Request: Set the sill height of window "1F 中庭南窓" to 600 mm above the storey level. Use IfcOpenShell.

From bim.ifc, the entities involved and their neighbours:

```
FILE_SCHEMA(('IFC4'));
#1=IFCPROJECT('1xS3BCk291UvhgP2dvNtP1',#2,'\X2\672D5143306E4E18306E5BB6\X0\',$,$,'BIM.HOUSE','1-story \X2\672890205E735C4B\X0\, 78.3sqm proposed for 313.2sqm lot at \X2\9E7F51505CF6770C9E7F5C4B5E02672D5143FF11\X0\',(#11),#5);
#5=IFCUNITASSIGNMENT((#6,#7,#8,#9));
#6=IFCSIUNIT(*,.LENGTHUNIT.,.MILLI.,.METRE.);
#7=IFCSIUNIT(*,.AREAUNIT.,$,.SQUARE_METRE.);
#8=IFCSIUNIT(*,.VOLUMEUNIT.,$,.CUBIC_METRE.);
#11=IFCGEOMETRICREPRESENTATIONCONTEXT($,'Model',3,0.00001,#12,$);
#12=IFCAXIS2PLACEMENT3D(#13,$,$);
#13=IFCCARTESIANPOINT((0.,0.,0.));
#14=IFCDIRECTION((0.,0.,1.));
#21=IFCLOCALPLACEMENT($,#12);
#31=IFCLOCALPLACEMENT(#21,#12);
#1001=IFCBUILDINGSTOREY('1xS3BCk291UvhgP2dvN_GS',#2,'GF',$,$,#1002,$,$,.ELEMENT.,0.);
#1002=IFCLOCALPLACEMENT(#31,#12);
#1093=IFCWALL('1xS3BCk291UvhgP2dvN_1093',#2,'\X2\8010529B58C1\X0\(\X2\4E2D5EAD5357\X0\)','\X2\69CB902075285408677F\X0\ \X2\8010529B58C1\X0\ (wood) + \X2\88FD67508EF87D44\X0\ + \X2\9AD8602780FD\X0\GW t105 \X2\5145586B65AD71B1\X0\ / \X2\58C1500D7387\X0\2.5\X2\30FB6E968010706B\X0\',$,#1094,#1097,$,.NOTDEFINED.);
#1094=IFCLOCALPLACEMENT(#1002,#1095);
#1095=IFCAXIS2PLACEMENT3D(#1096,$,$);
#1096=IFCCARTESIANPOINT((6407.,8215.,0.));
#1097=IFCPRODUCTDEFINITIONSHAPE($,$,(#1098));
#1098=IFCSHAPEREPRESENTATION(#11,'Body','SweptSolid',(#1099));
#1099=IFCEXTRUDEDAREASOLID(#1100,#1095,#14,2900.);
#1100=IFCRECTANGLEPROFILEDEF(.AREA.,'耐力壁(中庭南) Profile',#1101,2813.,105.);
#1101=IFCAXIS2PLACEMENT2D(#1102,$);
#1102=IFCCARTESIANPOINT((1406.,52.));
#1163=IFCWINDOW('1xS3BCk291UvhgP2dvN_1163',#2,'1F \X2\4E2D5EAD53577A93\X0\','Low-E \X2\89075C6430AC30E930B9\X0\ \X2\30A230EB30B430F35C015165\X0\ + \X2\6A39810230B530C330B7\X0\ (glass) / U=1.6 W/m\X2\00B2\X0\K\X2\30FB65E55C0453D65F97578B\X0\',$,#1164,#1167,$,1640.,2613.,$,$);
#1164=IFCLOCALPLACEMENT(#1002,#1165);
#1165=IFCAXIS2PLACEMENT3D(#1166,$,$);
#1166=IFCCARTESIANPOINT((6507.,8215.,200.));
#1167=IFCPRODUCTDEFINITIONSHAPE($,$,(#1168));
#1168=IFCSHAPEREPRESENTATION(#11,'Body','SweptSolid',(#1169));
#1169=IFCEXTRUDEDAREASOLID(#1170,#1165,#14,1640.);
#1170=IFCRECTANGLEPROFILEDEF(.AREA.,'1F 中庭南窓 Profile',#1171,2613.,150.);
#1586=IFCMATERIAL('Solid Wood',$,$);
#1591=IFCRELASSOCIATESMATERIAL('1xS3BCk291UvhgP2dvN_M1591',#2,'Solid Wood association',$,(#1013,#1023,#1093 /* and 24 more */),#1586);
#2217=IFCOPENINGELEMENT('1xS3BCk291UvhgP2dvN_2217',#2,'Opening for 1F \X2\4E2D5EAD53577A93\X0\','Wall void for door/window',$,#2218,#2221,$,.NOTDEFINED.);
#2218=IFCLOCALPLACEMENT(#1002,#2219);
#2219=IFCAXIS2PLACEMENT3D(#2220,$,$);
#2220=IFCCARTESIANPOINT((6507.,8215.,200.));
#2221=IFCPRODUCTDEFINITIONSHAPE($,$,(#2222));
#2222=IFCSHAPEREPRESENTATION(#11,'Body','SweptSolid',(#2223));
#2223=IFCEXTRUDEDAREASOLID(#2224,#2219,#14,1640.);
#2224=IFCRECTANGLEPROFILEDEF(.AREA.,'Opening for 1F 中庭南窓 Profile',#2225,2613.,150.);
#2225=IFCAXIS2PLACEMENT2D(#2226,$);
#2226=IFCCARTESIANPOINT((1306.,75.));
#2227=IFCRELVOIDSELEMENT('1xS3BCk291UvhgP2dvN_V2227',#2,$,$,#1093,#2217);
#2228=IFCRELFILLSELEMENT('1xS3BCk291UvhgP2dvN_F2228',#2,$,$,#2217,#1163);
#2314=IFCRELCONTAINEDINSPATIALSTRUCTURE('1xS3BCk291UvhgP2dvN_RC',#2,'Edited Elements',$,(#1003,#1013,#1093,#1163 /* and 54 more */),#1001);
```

```python
import numpy as np
import ifcopenshell
import ifcopenshell.api.geometry
import ifcopenshell.geom
import ifcopenshell.util.element
import ifcopenshell.util.placement
import ifcopenshell.util.shape
import ifcopenshell.util.unit

model = ifcopenshell.open("bim.ifc")
unit_scale = ifcopenshell.util.unit.calculate_unit_scale(model)

window = model.by_guid("1xS3BCk291UvhgP2dvN_1163")
opening = window.FillsVoids[0].RelatingOpeningElement
storey = ifcopenshell.util.element.get_container(window, ifc_class="IfcBuildingStorey")
level = ifcopenshell.util.placement.get_local_placement(storey.ObjectPlacement)[2, 3]

# The opening's origin need not be at the sill, so measure its lowest point.
shape = ifcopenshell.geom.create_shape(ifcopenshell.geom.settings(), opening)
bottom = ifcopenshell.util.shape.get_shape_bottom_elevation(shape, shape.geometry) / unit_scale
dz = level + 600.0 - bottom

shift = np.array([0.0, 0.0, dz])
# The window is not placed relative to its opening, so move both.
for product in (opening, window):
    matrix = ifcopenshell.util.placement.get_local_placement(product.ObjectPlacement)
    matrix[:3, 3] += shift
    ifcopenshell.api.geometry.edit_object_placement(model, product=product, matrix=matrix, is_si=False)

print(f"moved by {dz * unit_scale:+.3f} m")

model.write("bim_rev.ifc")
```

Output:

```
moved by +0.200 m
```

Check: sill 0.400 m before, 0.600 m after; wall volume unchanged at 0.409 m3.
